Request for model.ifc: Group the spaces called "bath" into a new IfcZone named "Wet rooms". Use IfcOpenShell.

First a look at what the model holds.

```python
import ifcopenshell

model = ifcopenshell.open("model.ifc")
print(model.schema)
seen = {}
for space in model.by_type("IfcSpace"):
    seen[space.LongName] = seen.get(space.LongName, 0) + 1
for name, count in sorted(seen.items(), key=str):
    print(count, "x", name)
print("zones:", [z.Name for z in model.by_type("IfcZone")][:20])
```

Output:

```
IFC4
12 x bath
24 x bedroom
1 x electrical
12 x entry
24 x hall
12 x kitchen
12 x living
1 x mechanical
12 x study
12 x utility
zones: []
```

```python
import ifcopenshell
import ifcopenshell.api.group
import ifcopenshell.api.root

model = ifcopenshell.open("model.ifc")

names = {"bath"}
spaces = [s for s in model.by_type("IfcSpace") if s.LongName in names]

zone = ifcopenshell.api.root.create_entity(model, ifc_class="IfcZone", name="Wet rooms")
ifcopenshell.api.group.assign_group(model, products=spaces, group=zone)
print(len(spaces), "spaces in", zone.Name)

model.write("model_v2.ifc")
```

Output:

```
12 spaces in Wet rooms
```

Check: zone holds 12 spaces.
